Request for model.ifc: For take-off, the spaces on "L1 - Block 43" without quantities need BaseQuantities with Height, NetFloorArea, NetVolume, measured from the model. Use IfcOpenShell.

First a look at what the model holds.

```python
import ifcopenshell
import ifcopenshell.util.element
import ifcopenshell.util.unit

model = ifcopenshell.open("model.ifc")
print(model.schema)
for unit_type in ("LENGTHUNIT", "AREAUNIT", "VOLUMEUNIT"):
    print(unit_type, ifcopenshell.util.unit.calculate_unit_scale(model, unit_type))
storey = next(s for s in model.by_type("IfcBuildingStorey") if s.Name == "L1 - Block 43")
spaces = [e for e in ifcopenshell.util.element.get_decomposition(storey) if e.is_a("IfcSpace")]
for e in sorted(spaces, key=lambda e: e.id()):
    print(e.id(), e.is_a(), e.Name, list(ifcopenshell.util.element.get_psets(e, qtos_only=True)), sep=" | ")
```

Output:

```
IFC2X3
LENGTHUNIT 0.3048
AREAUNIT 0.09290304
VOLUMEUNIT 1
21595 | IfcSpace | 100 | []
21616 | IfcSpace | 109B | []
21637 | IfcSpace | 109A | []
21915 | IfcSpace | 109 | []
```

```python
import ifcopenshell
import ifcopenshell.api.pset
import ifcopenshell.geom
import ifcopenshell.util.element
import ifcopenshell.util.shape
import ifcopenshell.util.unit

model = ifcopenshell.open("model.ifc")
unit_scale = ifcopenshell.util.unit.calculate_unit_scale(model)
area_scale = ifcopenshell.util.unit.calculate_unit_scale(model, "AREAUNIT")
volume_scale = ifcopenshell.util.unit.calculate_unit_scale(model, "VOLUMEUNIT")
settings = ifcopenshell.geom.settings()

storey = next(s for s in model.by_type("IfcBuildingStorey") if s.Name == "L1 - Block 43")
spaces = [e for e in ifcopenshell.util.element.get_decomposition(storey) if e.is_a("IfcSpace")]

for e in sorted(spaces, key=lambda e: e.id()):
    if ifcopenshell.util.element.get_psets(e, qtos_only=True, should_inherit=False):
        continue
    # Geometry comes back in metres, in the element's own axes.
    shape = ifcopenshell.geom.create_shape(settings, e)
    values = {
        "Height": ifcopenshell.util.shape.get_z(shape.geometry) / unit_scale,
        "NetFloorArea": ifcopenshell.util.shape.get_footprint_area(shape.geometry) / area_scale,
        "NetVolume": ifcopenshell.util.shape.get_volume(shape.geometry) / volume_scale,
    }
    qto = ifcopenshell.api.pset.add_qto(model, product=e, name="BaseQuantities")
    ifcopenshell.api.pset.edit_qto(model, qto=qto, properties=values)
    print(e.id(), {k: round(v, 3) for k, v in values.items()})

model.write("model-out.ifc")
```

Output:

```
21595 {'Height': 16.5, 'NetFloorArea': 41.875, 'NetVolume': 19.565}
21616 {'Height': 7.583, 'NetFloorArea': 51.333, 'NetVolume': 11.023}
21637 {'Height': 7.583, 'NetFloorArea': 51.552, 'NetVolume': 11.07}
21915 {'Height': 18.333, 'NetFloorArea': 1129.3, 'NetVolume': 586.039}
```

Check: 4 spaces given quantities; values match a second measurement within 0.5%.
